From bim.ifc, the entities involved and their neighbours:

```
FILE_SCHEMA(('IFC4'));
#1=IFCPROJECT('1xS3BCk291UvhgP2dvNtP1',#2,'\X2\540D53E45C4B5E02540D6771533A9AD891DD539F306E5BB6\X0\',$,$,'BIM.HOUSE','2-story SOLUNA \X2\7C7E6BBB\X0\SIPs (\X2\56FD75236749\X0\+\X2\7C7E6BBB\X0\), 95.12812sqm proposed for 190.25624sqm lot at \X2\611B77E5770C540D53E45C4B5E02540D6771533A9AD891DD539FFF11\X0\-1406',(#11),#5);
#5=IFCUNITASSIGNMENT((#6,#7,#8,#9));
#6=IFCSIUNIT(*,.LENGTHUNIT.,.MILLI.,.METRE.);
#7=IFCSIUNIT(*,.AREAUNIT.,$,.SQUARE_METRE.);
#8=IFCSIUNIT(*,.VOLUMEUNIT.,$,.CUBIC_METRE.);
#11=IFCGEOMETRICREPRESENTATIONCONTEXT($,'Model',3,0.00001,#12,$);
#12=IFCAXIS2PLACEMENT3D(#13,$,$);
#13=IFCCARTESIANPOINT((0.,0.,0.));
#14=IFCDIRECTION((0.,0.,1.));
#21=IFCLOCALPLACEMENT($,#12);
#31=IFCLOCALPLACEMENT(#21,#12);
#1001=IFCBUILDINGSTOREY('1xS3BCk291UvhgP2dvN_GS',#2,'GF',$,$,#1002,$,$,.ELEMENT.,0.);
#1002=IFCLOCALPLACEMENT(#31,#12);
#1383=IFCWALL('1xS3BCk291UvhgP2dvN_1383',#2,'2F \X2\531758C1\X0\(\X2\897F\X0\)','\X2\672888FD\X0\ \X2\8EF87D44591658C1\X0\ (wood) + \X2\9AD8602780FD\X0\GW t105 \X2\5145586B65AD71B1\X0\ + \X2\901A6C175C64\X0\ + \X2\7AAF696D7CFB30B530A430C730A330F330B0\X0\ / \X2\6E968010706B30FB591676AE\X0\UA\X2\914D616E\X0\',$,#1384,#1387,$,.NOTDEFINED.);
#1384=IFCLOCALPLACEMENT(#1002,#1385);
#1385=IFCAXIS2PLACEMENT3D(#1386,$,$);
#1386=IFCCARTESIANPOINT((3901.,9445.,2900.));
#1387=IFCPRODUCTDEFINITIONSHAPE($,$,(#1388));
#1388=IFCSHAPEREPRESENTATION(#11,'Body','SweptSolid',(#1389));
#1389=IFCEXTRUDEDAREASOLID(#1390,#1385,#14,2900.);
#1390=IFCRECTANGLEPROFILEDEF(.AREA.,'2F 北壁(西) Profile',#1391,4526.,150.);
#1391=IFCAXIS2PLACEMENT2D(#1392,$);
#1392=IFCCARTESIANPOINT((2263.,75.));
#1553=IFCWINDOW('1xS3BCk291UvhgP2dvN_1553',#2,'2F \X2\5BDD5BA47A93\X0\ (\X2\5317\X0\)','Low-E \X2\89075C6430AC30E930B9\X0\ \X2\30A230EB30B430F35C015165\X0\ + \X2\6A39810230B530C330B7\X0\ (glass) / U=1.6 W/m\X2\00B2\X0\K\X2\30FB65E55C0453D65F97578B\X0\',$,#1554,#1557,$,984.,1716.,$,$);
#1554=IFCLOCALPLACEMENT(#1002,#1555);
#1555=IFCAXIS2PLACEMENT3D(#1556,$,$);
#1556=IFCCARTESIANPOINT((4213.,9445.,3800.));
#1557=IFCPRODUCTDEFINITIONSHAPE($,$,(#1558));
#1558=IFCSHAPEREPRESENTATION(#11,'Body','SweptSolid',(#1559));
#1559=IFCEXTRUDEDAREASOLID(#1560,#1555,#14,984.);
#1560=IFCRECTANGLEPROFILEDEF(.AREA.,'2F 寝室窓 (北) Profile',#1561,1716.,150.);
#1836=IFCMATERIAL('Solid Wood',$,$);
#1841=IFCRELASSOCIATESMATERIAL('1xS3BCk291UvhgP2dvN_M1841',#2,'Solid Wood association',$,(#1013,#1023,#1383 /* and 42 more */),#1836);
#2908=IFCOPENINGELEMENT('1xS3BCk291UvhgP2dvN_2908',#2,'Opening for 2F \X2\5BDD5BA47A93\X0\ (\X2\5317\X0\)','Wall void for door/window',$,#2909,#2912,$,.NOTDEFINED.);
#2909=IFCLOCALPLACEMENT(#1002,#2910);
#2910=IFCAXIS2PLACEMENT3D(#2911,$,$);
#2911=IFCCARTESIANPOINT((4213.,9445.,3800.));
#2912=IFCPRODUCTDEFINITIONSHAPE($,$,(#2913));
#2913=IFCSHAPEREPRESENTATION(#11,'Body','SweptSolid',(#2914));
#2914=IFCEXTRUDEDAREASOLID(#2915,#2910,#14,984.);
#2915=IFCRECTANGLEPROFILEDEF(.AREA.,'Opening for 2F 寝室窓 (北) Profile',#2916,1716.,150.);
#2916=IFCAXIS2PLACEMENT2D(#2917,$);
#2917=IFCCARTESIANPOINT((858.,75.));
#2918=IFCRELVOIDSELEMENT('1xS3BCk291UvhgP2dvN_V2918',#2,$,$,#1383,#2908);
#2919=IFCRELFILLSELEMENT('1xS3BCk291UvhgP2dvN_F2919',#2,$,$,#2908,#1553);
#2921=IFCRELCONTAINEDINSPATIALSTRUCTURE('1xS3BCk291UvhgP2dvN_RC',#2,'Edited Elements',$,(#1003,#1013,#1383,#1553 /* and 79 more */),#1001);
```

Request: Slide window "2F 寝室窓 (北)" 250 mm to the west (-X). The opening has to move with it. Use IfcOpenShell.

```python
import ifcopenshell
import ifcopenshell.api.geometry
import ifcopenshell.util.placement

model = ifcopenshell.open("bim.ifc")

window = model.by_id(1553)
opening = window.FillsVoids[0].RelatingOpeningElement
wall = opening.VoidsElements[0].RelatingBuildingElement

wall_matrix = ifcopenshell.util.placement.get_local_placement(wall.ObjectPlacement)
shift = wall_matrix[:3, 0] * -250.0
before = ifcopenshell.util.placement.get_local_placement(window.ObjectPlacement)[:3, 3].copy()

# The window is not placed relative to its opening, so move both.
for product in (opening, window):
    matrix = ifcopenshell.util.placement.get_local_placement(product.ObjectPlacement)
    matrix[:3, 3] += shift
    ifcopenshell.api.geometry.edit_object_placement(model, product=product, matrix=matrix, is_si=False)

after = ifcopenshell.util.placement.get_local_placement(window.ObjectPlacement)[:3, 3]
print("window moved by", (after - before).round(3) + 0.0)

model.write("bim-out.ifc")
```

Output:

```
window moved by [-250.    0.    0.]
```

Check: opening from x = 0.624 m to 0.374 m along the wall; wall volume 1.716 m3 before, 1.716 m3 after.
